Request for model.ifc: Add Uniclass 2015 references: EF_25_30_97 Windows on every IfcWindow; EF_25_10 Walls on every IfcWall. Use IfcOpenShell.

First a look at what the model holds.

```python
import ifcopenshell

model = ifcopenshell.open("model.ifc")
print(model.schema)
print("classifications:", [c.Name for c in model.by_type("IfcClassification")])
for ifc_class in ("IfcDoor", "IfcRoof", "IfcStair", "IfcWall", "IfcWindow"):
    print(ifc_class, len(model.by_type(ifc_class)))
```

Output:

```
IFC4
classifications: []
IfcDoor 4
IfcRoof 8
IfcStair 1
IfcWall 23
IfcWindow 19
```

```python
import ifcopenshell
import ifcopenshell.api.classification

model = ifcopenshell.open("model.ifc")

system = ifcopenshell.api.classification.add_classification(model, classification="Uniclass 2015")

codes = {
    "IfcWindow": ("EF_25_30_97", "Windows"),
    "IfcWall": ("EF_25_10", "Walls"),
}
for ifc_class, (code, name) in codes.items():
    products = model.by_type(ifc_class)
    ifcopenshell.api.classification.add_reference(
        model, products=products, classification=system, identification=code, name=name
    )
    print(code, len(products))

model.write("model_v2.ifc")
```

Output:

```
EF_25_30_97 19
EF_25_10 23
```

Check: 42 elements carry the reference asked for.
